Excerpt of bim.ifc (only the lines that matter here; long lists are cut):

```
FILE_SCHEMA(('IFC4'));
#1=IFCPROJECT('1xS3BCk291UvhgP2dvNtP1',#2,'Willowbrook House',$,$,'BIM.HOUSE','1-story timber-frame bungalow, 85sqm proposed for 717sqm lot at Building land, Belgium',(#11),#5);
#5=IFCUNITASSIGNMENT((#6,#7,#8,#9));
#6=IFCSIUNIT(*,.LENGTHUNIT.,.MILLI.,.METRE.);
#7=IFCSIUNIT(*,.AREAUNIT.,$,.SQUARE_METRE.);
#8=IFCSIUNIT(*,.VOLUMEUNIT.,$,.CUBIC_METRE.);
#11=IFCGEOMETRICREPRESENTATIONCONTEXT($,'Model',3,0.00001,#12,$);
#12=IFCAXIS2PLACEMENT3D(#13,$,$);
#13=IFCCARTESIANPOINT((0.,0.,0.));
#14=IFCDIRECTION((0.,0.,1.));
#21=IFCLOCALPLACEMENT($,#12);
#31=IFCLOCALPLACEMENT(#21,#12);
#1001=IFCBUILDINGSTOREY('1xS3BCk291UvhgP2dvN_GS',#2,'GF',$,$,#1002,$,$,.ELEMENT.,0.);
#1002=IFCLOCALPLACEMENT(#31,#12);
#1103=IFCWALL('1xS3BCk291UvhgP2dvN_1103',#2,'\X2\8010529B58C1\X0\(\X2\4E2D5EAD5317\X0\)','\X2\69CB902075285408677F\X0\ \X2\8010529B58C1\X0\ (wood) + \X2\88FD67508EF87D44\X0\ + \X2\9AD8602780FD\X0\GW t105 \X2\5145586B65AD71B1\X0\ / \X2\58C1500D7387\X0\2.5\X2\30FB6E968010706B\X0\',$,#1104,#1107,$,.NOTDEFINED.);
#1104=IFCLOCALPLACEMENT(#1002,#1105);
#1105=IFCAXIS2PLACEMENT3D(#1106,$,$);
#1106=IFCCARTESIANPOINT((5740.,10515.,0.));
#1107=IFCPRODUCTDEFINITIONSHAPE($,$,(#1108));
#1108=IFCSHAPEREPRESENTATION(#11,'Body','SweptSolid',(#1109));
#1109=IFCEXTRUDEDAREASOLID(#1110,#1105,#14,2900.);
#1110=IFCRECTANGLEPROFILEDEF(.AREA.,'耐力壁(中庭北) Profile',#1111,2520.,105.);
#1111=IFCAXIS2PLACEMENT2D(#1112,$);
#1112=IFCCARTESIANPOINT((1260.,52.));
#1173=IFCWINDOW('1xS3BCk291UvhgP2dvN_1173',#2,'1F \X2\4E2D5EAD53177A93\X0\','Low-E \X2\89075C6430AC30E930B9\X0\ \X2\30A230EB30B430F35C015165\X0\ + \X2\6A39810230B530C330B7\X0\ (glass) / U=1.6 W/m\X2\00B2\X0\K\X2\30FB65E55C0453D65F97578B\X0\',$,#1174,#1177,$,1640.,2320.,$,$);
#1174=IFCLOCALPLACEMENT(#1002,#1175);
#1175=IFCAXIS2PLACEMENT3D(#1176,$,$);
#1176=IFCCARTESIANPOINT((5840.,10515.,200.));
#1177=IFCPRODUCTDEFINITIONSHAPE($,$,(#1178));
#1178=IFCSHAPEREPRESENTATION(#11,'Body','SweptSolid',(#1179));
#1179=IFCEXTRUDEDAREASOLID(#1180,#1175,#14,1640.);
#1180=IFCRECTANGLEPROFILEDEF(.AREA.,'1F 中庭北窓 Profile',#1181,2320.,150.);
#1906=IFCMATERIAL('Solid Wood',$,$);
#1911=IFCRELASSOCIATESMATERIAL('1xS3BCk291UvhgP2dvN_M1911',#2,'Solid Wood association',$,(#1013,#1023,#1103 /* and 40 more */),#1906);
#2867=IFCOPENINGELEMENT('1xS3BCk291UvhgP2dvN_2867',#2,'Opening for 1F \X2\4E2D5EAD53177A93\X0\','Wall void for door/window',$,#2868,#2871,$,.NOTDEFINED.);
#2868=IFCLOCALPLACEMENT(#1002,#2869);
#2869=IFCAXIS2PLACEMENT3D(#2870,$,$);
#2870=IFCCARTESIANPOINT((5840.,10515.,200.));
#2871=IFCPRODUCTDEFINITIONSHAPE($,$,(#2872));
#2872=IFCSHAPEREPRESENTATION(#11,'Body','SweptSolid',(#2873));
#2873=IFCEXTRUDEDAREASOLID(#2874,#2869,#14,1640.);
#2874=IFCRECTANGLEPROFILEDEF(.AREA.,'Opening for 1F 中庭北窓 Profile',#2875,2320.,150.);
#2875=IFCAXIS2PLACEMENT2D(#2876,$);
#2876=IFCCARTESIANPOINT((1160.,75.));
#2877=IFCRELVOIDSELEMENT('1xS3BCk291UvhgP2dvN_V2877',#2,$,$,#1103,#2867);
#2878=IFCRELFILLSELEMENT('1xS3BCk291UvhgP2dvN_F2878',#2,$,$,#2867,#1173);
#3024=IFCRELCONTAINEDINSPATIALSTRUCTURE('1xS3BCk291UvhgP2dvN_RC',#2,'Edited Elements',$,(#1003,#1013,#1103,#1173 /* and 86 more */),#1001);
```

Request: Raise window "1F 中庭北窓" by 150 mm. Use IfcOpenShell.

```python
import numpy as np
import ifcopenshell
import ifcopenshell.api.geometry
import ifcopenshell.util.placement
import ifcopenshell.util.unit

model = ifcopenshell.open("bim.ifc")
unit_scale = ifcopenshell.util.unit.calculate_unit_scale(model)

window = model.by_id(1173)
opening = window.FillsVoids[0].RelatingOpeningElement
dz = 0.15 / unit_scale

shift = np.array([0.0, 0.0, dz])
# The window is not placed relative to its opening, so move both.
for product in (opening, window):
    matrix = ifcopenshell.util.placement.get_local_placement(product.ObjectPlacement)
    matrix[:3, 3] += shift
    ifcopenshell.api.geometry.edit_object_placement(model, product=product, matrix=matrix, is_si=False)

print(f"moved by {dz * unit_scale:+.3f} m")

model.write("bim-out.ifc")
```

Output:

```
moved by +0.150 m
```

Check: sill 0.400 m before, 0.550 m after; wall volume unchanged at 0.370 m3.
